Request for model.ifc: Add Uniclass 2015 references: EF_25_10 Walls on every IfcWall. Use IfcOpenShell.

First a look at what the model holds.

```python
import ifcopenshell

model = ifcopenshell.open("model.ifc")
print(model.schema)
print("classifications:", [c.Name for c in model.by_type("IfcClassification")])
for ifc_class in ("IfcDoor", "IfcRoof", "IfcStair", "IfcWall", "IfcWindow"):
    print(ifc_class, len(model.by_type(ifc_class)))
```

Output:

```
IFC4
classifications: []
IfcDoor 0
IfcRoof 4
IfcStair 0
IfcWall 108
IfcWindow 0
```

```python
import ifcopenshell
import ifcopenshell.api.classification

model = ifcopenshell.open("model.ifc")

system = ifcopenshell.api.classification.add_classification(model, classification="Uniclass 2015")

codes = {
    "IfcWall": ("EF_25_10", "Walls"),
}
for ifc_class, (code, name) in codes.items():
    products = model.by_type(ifc_class)
    ifcopenshell.api.classification.add_reference(
        model, products=products, classification=system, identification=code, name=name
    )
    print(code, len(products))

model.write("model_edited.ifc")
```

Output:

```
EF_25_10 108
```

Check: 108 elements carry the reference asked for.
